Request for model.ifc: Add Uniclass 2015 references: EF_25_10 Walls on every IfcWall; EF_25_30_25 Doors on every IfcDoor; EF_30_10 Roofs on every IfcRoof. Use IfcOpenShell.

First a look at what the model holds.

```python
import ifcopenshell

model = ifcopenshell.open("model.ifc")
print(model.schema)
print("classifications:", [c.Name for c in model.by_type("IfcClassification")])
for ifc_class in ("IfcDoor", "IfcRoof", "IfcStair", "IfcWall", "IfcWindow"):
    print(ifc_class, len(model.by_type(ifc_class)))
```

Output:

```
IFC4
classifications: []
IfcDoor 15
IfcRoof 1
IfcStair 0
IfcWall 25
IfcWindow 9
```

```python
import ifcopenshell
import ifcopenshell.api.classification

model = ifcopenshell.open("model.ifc")

system = ifcopenshell.api.classification.add_classification(model, classification="Uniclass 2015")

codes = {
    "IfcWall": ("EF_25_10", "Walls"),
    "IfcDoor": ("EF_25_30_25", "Doors"),
    "IfcRoof": ("EF_30_10", "Roofs"),
}
for ifc_class, (code, name) in codes.items():
    products = model.by_type(ifc_class)
    ifcopenshell.api.classification.add_reference(
        model, products=products, classification=system, identification=code, name=name
    )
    print(code, len(products))

model.write("model_v2.ifc")
```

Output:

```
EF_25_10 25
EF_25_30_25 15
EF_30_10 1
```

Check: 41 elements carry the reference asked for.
